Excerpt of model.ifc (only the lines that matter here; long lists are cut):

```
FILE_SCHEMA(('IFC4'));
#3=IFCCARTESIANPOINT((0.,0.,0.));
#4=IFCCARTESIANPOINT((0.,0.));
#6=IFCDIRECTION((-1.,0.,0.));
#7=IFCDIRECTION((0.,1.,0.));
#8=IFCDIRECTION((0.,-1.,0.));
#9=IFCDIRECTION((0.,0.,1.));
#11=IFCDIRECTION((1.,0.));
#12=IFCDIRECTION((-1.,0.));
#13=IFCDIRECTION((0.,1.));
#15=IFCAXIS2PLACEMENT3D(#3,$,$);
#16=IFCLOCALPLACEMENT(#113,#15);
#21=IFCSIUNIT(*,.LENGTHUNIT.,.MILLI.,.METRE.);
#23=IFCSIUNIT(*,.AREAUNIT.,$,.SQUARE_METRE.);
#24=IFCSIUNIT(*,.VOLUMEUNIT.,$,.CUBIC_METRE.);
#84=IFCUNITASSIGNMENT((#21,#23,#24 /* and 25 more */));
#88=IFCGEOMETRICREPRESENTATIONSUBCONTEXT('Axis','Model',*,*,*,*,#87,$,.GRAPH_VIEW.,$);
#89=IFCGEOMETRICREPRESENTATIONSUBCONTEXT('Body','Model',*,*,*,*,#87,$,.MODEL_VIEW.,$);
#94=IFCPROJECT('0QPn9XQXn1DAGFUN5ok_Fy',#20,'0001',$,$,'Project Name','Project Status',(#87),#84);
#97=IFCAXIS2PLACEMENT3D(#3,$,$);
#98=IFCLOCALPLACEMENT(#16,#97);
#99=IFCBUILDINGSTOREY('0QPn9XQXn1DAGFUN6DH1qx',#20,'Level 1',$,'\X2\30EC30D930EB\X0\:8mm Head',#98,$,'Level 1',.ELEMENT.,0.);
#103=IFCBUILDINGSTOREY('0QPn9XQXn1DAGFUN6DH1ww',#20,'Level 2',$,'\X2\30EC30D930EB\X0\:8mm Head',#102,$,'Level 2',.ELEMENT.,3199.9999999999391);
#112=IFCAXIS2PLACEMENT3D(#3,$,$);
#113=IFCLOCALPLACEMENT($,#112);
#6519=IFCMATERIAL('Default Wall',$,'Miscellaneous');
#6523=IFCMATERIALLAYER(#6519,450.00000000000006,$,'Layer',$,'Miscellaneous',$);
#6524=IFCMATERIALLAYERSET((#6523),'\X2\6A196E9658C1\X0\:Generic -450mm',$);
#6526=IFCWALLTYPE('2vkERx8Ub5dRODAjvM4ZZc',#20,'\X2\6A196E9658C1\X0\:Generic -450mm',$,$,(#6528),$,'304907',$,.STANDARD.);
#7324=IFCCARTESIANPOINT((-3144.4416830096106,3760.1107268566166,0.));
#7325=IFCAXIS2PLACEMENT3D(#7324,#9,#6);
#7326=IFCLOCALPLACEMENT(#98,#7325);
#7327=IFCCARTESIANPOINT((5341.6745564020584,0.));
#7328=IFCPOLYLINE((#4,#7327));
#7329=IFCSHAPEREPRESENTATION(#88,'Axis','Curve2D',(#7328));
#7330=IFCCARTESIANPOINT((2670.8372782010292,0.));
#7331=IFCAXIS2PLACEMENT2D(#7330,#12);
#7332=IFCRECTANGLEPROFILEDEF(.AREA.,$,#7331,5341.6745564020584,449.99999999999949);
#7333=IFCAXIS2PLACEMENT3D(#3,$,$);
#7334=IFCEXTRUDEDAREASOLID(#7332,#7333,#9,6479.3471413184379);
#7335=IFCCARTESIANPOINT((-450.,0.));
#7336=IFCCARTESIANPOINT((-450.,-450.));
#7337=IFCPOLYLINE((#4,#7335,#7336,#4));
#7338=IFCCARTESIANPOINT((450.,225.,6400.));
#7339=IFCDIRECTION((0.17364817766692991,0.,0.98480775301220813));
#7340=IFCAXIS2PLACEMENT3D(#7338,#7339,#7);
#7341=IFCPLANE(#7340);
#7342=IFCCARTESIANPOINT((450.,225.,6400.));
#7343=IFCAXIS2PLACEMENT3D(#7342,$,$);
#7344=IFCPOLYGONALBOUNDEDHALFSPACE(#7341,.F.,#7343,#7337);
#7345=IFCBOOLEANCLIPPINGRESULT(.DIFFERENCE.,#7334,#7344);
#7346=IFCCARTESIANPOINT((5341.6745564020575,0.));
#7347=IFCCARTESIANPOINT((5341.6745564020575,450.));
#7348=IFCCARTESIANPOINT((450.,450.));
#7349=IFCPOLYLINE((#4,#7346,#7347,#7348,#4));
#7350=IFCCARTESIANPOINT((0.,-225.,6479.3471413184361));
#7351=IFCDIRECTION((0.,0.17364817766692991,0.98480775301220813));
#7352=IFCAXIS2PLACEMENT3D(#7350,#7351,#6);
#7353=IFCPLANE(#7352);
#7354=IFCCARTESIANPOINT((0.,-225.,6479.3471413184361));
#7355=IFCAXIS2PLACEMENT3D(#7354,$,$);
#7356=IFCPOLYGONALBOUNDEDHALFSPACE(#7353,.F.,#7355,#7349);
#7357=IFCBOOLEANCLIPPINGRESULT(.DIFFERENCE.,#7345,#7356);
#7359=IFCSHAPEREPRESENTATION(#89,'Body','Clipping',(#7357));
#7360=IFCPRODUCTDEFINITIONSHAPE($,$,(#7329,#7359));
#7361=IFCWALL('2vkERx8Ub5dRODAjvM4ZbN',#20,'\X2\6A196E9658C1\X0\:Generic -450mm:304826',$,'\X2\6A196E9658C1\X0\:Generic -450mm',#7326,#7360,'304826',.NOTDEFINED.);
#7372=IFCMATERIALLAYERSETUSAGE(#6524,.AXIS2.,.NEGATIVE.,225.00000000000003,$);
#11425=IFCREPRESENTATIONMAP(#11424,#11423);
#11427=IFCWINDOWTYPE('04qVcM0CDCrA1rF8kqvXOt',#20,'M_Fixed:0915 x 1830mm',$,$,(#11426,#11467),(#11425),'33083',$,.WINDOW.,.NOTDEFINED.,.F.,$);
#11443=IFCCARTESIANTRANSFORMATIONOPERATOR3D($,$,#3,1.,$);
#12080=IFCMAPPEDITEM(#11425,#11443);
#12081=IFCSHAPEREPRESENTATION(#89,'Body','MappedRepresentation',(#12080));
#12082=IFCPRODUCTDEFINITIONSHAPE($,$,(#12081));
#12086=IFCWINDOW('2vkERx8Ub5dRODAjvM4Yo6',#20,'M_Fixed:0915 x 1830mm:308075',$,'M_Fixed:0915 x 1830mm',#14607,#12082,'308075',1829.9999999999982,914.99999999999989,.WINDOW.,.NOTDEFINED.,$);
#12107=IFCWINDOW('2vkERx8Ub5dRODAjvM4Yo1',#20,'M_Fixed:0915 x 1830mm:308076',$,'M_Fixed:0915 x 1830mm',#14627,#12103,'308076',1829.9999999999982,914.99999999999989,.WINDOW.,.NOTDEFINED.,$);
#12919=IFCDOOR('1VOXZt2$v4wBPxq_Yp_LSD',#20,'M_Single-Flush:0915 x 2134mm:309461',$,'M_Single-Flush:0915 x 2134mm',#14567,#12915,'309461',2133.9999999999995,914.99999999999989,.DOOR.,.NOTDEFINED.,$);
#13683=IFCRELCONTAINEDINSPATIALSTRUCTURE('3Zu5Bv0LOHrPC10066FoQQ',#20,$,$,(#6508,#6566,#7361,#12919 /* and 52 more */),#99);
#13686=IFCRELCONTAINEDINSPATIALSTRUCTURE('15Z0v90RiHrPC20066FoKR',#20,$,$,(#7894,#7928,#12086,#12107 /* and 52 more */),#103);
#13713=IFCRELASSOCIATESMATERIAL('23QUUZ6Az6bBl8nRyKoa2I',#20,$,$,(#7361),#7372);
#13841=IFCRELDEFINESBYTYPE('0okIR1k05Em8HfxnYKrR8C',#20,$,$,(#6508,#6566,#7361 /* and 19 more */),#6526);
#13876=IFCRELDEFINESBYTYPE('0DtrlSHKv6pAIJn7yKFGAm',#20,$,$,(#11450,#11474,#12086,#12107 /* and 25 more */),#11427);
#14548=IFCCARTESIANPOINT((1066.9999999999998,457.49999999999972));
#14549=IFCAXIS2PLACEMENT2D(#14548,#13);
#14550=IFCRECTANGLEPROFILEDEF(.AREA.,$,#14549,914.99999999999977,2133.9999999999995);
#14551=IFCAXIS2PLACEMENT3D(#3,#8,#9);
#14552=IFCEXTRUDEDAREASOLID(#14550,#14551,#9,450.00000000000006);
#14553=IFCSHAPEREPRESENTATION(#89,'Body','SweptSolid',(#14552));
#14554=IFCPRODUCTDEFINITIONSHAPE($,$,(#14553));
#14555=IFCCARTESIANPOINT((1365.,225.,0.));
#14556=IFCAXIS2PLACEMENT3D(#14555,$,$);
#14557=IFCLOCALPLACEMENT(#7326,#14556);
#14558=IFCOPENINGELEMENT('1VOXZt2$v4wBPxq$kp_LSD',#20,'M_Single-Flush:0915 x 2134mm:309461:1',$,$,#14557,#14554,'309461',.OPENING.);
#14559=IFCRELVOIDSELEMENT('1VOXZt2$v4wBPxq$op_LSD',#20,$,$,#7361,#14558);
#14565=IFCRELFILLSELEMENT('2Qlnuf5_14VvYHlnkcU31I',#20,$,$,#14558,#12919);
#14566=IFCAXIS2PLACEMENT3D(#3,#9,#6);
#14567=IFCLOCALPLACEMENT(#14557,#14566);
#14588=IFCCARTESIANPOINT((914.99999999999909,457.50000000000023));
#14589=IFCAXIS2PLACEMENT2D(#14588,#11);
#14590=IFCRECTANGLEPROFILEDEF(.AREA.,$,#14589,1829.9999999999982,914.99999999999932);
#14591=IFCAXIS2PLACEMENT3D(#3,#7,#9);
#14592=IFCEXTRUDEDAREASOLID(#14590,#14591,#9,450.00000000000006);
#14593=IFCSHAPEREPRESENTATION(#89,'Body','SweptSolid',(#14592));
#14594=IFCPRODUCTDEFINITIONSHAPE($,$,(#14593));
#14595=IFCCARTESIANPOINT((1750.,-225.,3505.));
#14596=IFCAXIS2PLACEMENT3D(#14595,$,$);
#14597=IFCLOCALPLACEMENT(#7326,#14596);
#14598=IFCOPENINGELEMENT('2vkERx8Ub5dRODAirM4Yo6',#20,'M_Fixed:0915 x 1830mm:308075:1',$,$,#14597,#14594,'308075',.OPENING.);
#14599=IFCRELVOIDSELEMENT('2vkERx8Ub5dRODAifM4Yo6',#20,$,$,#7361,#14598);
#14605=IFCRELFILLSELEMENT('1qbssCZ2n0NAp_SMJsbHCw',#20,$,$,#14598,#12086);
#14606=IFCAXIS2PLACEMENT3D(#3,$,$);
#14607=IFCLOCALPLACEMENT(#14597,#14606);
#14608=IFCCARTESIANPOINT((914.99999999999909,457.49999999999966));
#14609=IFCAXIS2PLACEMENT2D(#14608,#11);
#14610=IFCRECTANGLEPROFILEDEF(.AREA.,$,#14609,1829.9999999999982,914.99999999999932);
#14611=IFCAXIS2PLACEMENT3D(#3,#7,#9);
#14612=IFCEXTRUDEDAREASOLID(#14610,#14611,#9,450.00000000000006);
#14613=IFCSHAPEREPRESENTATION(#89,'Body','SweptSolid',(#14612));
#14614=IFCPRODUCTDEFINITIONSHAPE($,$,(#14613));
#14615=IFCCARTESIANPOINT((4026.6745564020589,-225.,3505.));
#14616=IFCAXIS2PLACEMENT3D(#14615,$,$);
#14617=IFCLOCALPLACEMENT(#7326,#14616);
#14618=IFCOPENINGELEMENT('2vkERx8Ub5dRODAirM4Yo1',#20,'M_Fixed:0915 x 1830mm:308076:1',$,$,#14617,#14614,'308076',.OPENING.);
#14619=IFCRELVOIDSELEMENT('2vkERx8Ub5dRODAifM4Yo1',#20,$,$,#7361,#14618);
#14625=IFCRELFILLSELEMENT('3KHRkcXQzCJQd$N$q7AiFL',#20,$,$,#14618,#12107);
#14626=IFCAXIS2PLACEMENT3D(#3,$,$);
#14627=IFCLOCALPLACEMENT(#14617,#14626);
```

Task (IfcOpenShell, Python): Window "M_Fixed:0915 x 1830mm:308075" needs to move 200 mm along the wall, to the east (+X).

```python
import ifcopenshell
import ifcopenshell.api.geometry
import ifcopenshell.util.placement
import ifcopenshell.util.unit

model = ifcopenshell.open("model.ifc")
unit_scale = ifcopenshell.util.unit.calculate_unit_scale(model)

window = model.by_id(12086)
opening = window.FillsVoids[0].RelatingOpeningElement
wall = opening.VoidsElements[0].RelatingBuildingElement

wall_matrix = ifcopenshell.util.placement.get_local_placement(wall.ObjectPlacement)
shift = wall_matrix[:3, 0] * -0.2 / unit_scale
before = ifcopenshell.util.placement.get_local_placement(window.ObjectPlacement)[:3, 3].copy()

# The window is placed relative to its opening, so it follows when the opening moves.
matrix = ifcopenshell.util.placement.get_local_placement(opening.ObjectPlacement)
matrix[:3, 3] += shift
ifcopenshell.api.geometry.edit_object_placement(
    model, product=opening, matrix=matrix, is_si=False, should_transform_children=True
)

after = ifcopenshell.util.placement.get_local_placement(window.ObjectPlacement)[:3, 3]
print("window moved by", (after - before).round(3) + 0.0)

model.write("model_updated.ifc")
```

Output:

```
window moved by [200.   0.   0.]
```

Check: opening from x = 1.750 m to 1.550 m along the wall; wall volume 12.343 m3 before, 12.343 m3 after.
